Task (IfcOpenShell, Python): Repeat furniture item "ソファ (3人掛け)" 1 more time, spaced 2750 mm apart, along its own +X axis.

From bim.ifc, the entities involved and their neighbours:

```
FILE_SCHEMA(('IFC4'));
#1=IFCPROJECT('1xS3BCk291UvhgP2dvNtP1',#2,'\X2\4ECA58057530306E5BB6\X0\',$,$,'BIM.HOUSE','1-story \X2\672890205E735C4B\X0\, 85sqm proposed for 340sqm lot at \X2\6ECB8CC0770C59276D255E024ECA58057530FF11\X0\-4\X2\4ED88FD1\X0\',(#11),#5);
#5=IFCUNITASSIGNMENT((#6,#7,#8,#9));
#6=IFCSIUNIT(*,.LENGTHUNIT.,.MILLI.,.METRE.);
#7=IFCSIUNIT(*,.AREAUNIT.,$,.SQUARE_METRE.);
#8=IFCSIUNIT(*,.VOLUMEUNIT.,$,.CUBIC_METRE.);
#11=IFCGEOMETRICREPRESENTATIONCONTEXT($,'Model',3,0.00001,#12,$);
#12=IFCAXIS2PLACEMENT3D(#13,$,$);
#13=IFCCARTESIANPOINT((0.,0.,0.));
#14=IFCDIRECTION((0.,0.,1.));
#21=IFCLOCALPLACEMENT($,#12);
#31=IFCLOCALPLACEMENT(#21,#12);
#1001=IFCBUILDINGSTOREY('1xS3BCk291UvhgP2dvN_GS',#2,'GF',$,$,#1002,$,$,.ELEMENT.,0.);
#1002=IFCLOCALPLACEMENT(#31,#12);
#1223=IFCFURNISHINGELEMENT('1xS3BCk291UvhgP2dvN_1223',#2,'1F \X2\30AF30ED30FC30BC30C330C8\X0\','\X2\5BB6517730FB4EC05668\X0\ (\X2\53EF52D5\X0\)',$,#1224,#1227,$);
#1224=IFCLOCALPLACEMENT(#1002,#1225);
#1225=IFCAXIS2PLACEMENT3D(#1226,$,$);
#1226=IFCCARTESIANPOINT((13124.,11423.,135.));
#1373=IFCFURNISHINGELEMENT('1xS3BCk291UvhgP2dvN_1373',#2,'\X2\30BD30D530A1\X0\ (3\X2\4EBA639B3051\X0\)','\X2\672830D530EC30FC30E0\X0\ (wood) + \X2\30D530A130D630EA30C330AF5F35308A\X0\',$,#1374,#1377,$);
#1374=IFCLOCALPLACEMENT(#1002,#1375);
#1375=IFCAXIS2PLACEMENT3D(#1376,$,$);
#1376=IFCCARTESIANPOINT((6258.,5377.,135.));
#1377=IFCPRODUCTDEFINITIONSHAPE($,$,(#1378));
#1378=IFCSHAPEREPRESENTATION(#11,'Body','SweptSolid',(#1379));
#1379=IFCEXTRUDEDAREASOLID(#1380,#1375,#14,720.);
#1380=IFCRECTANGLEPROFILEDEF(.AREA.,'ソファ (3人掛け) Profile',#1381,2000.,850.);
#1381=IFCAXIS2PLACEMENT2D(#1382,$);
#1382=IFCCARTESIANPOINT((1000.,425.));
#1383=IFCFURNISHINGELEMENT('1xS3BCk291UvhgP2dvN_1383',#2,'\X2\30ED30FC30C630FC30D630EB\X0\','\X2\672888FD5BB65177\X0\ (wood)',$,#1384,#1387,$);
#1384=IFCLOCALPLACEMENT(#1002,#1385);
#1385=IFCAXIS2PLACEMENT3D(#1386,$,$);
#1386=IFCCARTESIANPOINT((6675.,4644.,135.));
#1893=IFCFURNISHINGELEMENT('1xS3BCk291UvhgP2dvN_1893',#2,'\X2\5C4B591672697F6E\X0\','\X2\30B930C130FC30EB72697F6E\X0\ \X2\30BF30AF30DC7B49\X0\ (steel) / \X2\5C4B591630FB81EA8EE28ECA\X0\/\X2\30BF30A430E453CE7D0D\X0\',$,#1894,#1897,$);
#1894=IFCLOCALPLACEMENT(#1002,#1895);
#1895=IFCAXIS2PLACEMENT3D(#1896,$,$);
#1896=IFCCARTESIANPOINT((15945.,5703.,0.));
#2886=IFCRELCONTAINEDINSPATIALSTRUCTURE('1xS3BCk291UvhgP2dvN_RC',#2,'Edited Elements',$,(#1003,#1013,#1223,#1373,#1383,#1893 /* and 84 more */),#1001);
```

```python
import ifcopenshell
import ifcopenshell.api.geometry
import ifcopenshell.api.root
import ifcopenshell.util.element
import ifcopenshell.util.placement

model = ifcopenshell.open("bim.ifc")


def reuse_history(source, copy):
    """copy_class also copies each property set's owner history, people and application; keep the originals."""
    for rel in copy.IsDefinedBy:
        if rel.is_a("IfcRelDefinesByProperties") and (history := rel.RelatingPropertyDefinition.OwnerHistory):
            rel.RelatingPropertyDefinition.OwnerHistory = source.OwnerHistory
            ifcopenshell.util.element.remove_deep2(model, history)


source = model.by_id(1373)
base = ifcopenshell.util.placement.get_local_placement(source.ObjectPlacement)
step = base[:3, 0] * 2750.0

for i in range(1, 2):
    copy = ifcopenshell.api.root.copy_class(model, product=source)
    copy.Representation = ifcopenshell.util.element.copy_deep(
        model, source.Representation, exclude=["IfcGeometricRepresentationContext", "IfcRepresentationMap"]
    )
    reuse_history(source, copy)
    matrix = base.copy()
    matrix[:3, 3] += i * step
    print("added at", matrix[:3, 3].round(3) + 0.0)
    ifcopenshell.api.geometry.edit_object_placement(model, product=copy, matrix=matrix, is_si=False)

model.write("bim_v2.ifc")
```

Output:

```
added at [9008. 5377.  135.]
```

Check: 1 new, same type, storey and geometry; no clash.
